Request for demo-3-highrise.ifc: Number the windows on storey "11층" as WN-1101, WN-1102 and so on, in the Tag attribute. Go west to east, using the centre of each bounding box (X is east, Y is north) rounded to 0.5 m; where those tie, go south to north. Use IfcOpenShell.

First a look at what the model holds.

```python
import ifcopenshell
import ifcopenshell.util.element
import ifcopenshell.util.placement

model = ifcopenshell.open("demo-3-highrise.ifc")
print(model.schema)
storey = next(s for s in model.by_type("IfcBuildingStorey") if s.Name == "11층")
windows = [e for e in ifcopenshell.util.element.get_decomposition(storey) if e.is_a("IfcWindow")]
for e in sorted(windows, key=lambda e: e.id()):
    origin = ifcopenshell.util.placement.get_local_placement(e.ObjectPlacement)[:3, 3]
    print(e.id(), e.Tag, e.Name, origin.round(2) + 0.0, sep=" | ")
```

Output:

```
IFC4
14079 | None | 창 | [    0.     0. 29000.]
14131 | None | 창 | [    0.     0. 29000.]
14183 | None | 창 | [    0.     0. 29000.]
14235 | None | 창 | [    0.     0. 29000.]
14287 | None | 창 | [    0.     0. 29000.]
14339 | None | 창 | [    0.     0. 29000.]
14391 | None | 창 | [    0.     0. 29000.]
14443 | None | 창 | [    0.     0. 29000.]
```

```python
import ifcopenshell
import ifcopenshell.geom
import ifcopenshell.util.element
import ifcopenshell.util.shape

model = ifcopenshell.open("demo-3-highrise.ifc")
settings = ifcopenshell.geom.settings()
settings.set("use-world-coords", True)


def centre(element):
    shape = ifcopenshell.geom.create_shape(settings, element)
    return ifcopenshell.util.shape.get_bbox_centroid(shape.geometry)


storey = next(s for s in model.by_type("IfcBuildingStorey") if s.Name == "11층")
windows = [e for e in ifcopenshell.util.element.get_decomposition(storey) if e.is_a("IfcWindow")]

# Insertion points can sit at a corner or the storey origin, so sort by the geometry (in metres).
centres = {e: centre(e) for e in windows}
windows.sort(key=lambda e: (round(centres[e][0] / 0.5), centres[e][1]))

for i, e in enumerate(windows, start=1):
    number = f"WN-11{i:02d}"
    e.Tag = number
    print(e.id(), number)

model.write("demo-3-highrise-out.ifc")
```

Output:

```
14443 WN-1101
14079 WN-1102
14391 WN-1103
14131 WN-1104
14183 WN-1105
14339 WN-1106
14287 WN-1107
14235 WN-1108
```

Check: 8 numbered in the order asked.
